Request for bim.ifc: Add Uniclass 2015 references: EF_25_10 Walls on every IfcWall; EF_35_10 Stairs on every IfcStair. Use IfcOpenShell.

First a look at what the model holds.

```python
import ifcopenshell

model = ifcopenshell.open("bim.ifc")
print(model.schema)
print("classifications:", [c.Name for c in model.by_type("IfcClassification")])
for ifc_class in ("IfcDoor", "IfcRoof", "IfcStair", "IfcWall", "IfcWindow"):
    print(ifc_class, len(model.by_type(ifc_class)))
```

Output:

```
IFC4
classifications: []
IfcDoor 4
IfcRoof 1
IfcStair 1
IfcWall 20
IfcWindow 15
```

```python
import ifcopenshell
import ifcopenshell.api.classification

model = ifcopenshell.open("bim.ifc")

system = ifcopenshell.api.classification.add_classification(model, classification="Uniclass 2015")

codes = {
    "IfcWall": ("EF_25_10", "Walls"),
    "IfcStair": ("EF_35_10", "Stairs"),
}
for ifc_class, (code, name) in codes.items():
    products = model.by_type(ifc_class)
    ifcopenshell.api.classification.add_reference(
        model, products=products, classification=system, identification=code, name=name
    )
    print(code, len(products))

model.write("bim_updated.ifc")
```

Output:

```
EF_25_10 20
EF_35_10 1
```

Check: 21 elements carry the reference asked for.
